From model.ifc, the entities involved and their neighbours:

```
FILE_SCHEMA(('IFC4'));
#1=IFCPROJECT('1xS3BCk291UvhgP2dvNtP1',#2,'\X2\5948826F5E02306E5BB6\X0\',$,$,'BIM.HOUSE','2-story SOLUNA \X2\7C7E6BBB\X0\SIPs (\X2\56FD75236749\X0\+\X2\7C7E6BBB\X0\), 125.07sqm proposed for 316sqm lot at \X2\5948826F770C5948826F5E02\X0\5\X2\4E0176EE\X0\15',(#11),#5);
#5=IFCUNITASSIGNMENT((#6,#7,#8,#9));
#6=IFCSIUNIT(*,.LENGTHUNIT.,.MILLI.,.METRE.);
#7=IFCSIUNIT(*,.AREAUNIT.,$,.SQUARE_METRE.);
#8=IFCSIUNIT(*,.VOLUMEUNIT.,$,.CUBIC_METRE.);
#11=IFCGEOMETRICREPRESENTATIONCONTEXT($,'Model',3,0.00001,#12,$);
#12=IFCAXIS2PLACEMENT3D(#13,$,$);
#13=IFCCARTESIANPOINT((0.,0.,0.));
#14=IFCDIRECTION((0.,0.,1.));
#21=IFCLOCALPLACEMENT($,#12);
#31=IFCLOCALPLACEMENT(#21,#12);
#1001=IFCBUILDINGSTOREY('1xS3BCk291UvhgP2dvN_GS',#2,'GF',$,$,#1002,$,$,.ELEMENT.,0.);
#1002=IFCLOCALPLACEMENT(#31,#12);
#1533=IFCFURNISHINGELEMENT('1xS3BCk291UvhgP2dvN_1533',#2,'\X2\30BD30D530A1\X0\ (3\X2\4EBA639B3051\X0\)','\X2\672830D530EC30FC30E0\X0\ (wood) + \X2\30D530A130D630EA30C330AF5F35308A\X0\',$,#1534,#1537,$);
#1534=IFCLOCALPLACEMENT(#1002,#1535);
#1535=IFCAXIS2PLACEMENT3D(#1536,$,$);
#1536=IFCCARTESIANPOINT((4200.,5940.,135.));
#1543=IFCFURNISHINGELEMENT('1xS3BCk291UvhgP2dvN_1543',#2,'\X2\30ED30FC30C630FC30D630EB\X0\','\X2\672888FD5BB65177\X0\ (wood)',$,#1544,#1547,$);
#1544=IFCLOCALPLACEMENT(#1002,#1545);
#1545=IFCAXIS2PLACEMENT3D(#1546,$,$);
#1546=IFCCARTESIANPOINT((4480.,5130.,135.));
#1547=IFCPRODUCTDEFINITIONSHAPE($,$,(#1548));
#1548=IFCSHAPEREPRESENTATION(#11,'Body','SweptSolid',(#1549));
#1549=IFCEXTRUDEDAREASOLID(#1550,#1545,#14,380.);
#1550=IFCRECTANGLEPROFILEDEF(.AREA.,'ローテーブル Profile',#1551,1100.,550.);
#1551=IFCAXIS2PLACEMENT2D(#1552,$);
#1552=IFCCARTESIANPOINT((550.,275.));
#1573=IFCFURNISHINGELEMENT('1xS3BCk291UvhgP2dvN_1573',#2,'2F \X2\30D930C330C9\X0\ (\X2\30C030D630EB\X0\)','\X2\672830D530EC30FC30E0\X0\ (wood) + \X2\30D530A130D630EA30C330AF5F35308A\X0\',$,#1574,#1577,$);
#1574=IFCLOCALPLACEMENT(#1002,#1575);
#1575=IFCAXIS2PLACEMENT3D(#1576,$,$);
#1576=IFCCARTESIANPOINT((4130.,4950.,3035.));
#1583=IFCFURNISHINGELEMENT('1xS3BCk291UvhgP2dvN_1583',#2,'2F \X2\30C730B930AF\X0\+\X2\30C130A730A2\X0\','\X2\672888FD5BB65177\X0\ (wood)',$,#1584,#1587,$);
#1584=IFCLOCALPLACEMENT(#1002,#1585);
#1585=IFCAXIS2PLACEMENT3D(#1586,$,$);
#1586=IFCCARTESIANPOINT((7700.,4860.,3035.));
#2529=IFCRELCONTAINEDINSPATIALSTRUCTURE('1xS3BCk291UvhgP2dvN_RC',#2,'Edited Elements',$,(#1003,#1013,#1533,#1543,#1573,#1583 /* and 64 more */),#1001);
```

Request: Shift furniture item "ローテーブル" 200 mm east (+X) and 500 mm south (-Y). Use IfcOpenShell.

```python
import ifcopenshell
import ifcopenshell.api.geometry
import ifcopenshell.util.placement

model = ifcopenshell.open("model.ifc")

item = model.by_id(1543)
matrix = ifcopenshell.util.placement.get_local_placement(item.ObjectPlacement)
matrix[0, 3] += 200.0
matrix[1, 3] -= 500.0
ifcopenshell.api.geometry.edit_object_placement(model, product=item, matrix=matrix, is_si=False)

print(ifcopenshell.util.placement.get_local_placement(item.ObjectPlacement).round(3) + 0.0)

model.write("model-out.ifc")
```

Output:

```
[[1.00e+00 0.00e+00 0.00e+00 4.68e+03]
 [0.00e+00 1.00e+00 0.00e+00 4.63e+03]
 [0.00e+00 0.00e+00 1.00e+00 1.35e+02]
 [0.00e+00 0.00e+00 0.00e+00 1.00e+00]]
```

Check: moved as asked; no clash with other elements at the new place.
